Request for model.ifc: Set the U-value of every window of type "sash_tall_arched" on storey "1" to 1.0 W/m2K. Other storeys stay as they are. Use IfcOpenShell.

First a look at what the model holds.

```python
import ifcopenshell
import ifcopenshell.util.element

model = ifcopenshell.open("model.ifc")
print(model.schema)
storey = next(s for s in model.by_type("IfcBuildingStorey") if s.Name == "1")
windows = [e for e in ifcopenshell.util.element.get_decomposition(storey) if e.is_a("IfcWindow")]
seen = {}
for e in windows:
    element_type = ifcopenshell.util.element.get_type(e)
    key = (element_type.Name if element_type != e and element_type else None, ifcopenshell.util.element.get_pset(e, "Pset_WindowCommon", "ThermalTransmittance"))
    seen[key] = seen.get(key, 0) + 1
for (name, value), count in sorted(seen.items(), key=str):
    print(count, "x", name, "|", value)
```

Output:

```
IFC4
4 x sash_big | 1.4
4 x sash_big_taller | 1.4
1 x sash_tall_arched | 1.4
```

```python
import ifcopenshell
import ifcopenshell.api.pset
import ifcopenshell.util.element

model = ifcopenshell.open("model.ifc")

storey = next(s for s in model.by_type("IfcBuildingStorey") if s.Name == "1")
windows = [e for e in ifcopenshell.util.element.get_decomposition(storey) if e.is_a("IfcWindow")]

count = 0
for e in windows:
    element_type = ifcopenshell.util.element.get_type(e)
    if element_type in (None, e) or element_type.Name != "sash_tall_arched":
        continue
    # add_pset returns the element's existing set when there is one.
    pset = ifcopenshell.api.pset.add_pset(model, product=e, name="Pset_WindowCommon")
    ifcopenshell.api.pset.edit_pset(model, pset=pset, properties={"ThermalTransmittance": 1.0})
    count += 1

print(count, "windows updated")

model.write("model_rev.ifc")
```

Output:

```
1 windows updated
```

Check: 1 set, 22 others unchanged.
